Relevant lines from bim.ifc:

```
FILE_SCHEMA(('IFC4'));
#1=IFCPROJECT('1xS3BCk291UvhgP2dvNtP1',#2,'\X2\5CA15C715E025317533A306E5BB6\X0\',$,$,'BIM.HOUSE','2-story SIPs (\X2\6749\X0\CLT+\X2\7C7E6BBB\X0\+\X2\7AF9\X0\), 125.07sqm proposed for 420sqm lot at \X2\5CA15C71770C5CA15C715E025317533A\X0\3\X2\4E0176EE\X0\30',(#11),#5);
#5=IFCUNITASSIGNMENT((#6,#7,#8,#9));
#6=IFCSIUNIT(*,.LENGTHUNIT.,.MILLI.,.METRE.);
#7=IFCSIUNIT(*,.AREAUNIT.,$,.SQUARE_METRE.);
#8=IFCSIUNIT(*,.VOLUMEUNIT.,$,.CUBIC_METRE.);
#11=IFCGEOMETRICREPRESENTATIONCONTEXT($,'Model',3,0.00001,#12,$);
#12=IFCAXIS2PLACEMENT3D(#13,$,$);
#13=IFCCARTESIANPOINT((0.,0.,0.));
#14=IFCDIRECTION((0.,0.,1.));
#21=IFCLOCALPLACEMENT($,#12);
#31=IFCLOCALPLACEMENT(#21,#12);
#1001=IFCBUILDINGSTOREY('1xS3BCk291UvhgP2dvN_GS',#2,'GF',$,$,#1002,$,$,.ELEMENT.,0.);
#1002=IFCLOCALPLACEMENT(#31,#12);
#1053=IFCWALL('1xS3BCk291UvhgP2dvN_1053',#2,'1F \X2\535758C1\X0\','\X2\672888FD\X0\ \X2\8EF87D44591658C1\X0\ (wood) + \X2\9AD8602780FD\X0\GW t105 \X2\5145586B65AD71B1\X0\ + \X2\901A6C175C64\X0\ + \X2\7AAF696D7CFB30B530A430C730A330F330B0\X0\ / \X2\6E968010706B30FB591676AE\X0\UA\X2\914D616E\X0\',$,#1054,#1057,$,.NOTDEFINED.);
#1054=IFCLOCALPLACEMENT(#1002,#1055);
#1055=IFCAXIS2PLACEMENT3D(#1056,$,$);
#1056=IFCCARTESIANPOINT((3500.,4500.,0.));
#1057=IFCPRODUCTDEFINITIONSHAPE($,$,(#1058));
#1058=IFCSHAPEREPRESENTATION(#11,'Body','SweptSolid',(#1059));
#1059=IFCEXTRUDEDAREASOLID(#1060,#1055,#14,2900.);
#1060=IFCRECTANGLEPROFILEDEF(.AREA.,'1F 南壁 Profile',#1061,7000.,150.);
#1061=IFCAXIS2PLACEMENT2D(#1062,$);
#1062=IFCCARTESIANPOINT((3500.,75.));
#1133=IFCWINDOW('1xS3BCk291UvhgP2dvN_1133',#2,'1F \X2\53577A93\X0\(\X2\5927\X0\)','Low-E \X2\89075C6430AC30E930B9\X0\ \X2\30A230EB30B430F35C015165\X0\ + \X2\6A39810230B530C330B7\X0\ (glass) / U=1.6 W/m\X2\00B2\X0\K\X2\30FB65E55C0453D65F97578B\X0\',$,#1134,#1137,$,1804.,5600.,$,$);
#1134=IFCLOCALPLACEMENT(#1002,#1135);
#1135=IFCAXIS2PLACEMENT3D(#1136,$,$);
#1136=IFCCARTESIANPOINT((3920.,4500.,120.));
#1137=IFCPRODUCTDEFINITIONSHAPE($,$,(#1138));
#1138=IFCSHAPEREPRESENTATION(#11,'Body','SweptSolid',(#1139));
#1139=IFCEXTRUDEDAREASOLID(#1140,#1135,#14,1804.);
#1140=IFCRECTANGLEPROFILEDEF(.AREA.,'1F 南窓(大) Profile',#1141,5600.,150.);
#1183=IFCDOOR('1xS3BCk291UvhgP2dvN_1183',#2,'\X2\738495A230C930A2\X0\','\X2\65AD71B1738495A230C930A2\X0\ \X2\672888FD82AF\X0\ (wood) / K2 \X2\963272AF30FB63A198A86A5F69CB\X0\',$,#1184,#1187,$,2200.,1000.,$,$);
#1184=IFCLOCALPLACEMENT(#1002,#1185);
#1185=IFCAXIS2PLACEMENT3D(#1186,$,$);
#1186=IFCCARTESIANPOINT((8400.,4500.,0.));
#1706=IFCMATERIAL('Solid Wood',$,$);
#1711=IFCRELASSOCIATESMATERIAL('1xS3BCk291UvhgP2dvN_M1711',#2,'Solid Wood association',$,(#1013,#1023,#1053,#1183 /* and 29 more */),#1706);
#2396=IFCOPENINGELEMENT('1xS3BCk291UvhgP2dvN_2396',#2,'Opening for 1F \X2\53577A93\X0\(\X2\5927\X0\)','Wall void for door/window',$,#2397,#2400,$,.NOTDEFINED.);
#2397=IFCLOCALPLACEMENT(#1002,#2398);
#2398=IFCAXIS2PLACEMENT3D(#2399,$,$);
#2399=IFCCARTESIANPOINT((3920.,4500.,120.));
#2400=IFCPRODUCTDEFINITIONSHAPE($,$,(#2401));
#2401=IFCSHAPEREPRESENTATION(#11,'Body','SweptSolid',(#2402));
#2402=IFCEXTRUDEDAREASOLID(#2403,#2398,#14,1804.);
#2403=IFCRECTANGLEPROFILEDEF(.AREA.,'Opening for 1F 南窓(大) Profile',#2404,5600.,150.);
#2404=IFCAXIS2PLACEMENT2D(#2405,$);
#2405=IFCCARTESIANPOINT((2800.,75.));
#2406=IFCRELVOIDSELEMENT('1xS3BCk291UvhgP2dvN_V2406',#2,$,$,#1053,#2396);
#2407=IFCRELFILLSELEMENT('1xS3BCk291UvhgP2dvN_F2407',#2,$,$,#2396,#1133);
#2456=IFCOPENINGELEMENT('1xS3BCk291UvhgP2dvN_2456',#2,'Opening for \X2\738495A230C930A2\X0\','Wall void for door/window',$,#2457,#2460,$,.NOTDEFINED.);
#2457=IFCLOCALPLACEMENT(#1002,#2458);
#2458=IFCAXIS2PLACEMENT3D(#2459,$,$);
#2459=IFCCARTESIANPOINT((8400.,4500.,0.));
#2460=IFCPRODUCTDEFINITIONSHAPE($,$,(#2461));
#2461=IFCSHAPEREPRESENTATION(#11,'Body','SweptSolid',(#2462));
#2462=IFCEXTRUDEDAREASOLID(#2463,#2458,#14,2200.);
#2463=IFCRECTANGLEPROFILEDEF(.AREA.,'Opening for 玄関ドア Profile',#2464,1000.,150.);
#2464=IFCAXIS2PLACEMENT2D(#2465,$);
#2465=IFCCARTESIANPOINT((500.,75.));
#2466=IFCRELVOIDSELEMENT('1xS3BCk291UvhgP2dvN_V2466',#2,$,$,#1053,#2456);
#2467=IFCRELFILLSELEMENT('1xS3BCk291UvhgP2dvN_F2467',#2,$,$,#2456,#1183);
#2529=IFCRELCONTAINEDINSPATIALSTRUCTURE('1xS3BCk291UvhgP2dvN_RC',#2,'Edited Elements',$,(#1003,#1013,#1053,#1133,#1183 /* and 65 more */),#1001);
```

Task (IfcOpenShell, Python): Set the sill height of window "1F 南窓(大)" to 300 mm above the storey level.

```python
import numpy as np
import ifcopenshell
import ifcopenshell.api.geometry
import ifcopenshell.geom
import ifcopenshell.util.element
import ifcopenshell.util.placement
import ifcopenshell.util.shape
import ifcopenshell.util.unit

model = ifcopenshell.open("bim.ifc")
unit_scale = ifcopenshell.util.unit.calculate_unit_scale(model)

window = model.by_id(1133)
opening = window.FillsVoids[0].RelatingOpeningElement
storey = ifcopenshell.util.element.get_container(window, ifc_class="IfcBuildingStorey")
level = ifcopenshell.util.placement.get_local_placement(storey.ObjectPlacement)[2, 3]

# The opening's origin need not be at the sill, so measure its lowest point.
shape = ifcopenshell.geom.create_shape(ifcopenshell.geom.settings(), opening)
bottom = ifcopenshell.util.shape.get_shape_bottom_elevation(shape, shape.geometry) / unit_scale
dz = level + 0.3 / unit_scale - bottom

shift = np.array([0.0, 0.0, dz])
# The window is not placed relative to its opening, so move both.
for product in (opening, window):
    matrix = ifcopenshell.util.placement.get_local_placement(product.ObjectPlacement)
    matrix[:3, 3] += shift
    ifcopenshell.api.geometry.edit_object_placement(model, product=product, matrix=matrix, is_si=False)

print(f"moved by {dz * unit_scale:+.3f} m")

model.write("bim_updated.ifc")
```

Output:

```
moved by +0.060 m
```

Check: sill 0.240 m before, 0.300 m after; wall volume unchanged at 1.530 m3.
